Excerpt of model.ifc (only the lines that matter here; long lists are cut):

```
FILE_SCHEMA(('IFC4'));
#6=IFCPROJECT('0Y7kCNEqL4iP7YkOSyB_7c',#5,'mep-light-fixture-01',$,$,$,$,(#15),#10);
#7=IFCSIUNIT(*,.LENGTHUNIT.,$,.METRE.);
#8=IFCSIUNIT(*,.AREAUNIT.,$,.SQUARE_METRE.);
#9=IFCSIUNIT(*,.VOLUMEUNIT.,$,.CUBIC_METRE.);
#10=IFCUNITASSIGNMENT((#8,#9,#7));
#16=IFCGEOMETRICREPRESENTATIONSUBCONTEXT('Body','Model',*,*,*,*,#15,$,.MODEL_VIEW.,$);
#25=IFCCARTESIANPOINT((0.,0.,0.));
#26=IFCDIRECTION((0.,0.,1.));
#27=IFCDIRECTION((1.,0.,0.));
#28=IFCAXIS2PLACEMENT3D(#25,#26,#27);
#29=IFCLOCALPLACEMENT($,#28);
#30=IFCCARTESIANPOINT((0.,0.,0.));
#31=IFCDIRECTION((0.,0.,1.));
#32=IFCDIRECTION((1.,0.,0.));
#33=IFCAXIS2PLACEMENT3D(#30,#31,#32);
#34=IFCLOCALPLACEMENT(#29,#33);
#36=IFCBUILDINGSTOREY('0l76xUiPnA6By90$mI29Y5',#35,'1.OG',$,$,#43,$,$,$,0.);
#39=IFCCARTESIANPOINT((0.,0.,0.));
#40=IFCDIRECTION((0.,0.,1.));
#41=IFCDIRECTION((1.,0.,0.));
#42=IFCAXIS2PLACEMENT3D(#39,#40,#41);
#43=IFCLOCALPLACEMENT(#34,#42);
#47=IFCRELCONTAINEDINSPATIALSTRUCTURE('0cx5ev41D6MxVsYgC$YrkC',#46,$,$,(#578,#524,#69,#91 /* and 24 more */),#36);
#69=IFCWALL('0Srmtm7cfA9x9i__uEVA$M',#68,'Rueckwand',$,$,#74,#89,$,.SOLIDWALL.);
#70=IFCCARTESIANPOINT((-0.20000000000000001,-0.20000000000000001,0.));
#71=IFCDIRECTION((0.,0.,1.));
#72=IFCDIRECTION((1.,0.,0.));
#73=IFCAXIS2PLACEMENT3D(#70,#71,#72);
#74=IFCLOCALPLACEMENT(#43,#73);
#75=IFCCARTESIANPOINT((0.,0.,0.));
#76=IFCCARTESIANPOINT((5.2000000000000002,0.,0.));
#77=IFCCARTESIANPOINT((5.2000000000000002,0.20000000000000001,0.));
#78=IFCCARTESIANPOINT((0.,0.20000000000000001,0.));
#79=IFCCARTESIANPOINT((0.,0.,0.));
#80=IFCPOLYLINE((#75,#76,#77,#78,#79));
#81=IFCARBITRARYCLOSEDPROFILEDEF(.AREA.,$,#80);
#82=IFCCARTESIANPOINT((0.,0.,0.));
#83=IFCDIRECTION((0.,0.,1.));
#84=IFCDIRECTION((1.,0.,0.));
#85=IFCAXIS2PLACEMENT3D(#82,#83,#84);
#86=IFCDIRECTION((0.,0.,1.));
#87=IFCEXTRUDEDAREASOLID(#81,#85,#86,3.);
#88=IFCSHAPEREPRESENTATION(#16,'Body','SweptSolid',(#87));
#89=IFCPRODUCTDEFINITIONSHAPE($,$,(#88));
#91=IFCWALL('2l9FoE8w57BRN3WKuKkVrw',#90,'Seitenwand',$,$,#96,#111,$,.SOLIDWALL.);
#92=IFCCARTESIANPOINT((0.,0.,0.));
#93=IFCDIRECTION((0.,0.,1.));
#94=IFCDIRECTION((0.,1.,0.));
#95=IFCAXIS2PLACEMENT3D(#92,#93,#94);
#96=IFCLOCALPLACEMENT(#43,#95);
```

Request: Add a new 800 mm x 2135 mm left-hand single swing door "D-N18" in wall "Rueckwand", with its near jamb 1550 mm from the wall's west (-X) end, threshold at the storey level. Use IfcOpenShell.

```python
import numpy as np
import ifcopenshell
import ifcopenshell.api.feature
import ifcopenshell.api.geometry
import ifcopenshell.api.root
import ifcopenshell.api.spatial
import ifcopenshell.geom
import ifcopenshell.util.element
import ifcopenshell.util.placement
import ifcopenshell.util.representation
import ifcopenshell.util.shape
import ifcopenshell.util.unit

model = ifcopenshell.open("model.ifc")
unit_scale = ifcopenshell.util.unit.calculate_unit_scale(model)
settings = ifcopenshell.geom.settings()


def volume(element):
    """Net volume in cubic metres, openings subtracted."""
    shape = ifcopenshell.geom.create_shape(settings, element)
    return ifcopenshell.util.shape.get_volume(shape.geometry)


wall = model.by_guid("0Srmtm7cfA9x9i__uEVA$M")
storey = ifcopenshell.util.element.get_container(wall, ifc_class="IfcBuildingStorey")
context = ifcopenshell.util.representation.get_context(model, "Model", "Body", "MODEL_VIEW")
before = volume(wall)

width, height, from_end, sill = 0.8, 2.135, 1.55, 0.0  # metres

# The wall runs along its own X axis, and the end named is its -X end.
wall_shape = ifcopenshell.geom.create_shape(settings, wall)
x, y, z = ifcopenshell.util.shape.get_vertices(wall_shape.geometry).T
start = x.min() + from_end
face, thickness = float(y.min()), float(y.max() - y.min())
wall_matrix = ifcopenshell.util.placement.get_local_placement(wall.ObjectPlacement)
level = ifcopenshell.util.placement.get_local_placement(storey.ObjectPlacement)[2, 3]


def in_wall(x, y):
    """Placement at x, y metres in the wall's axes, at sill height."""
    matrix = wall_matrix.copy()
    matrix[:, 3] = wall_matrix @ np.array([x / unit_scale, y / unit_scale, 0.0, 1.0])
    matrix[2, 3] = level + sill / unit_scale
    return matrix


# Opening: a box that overshoots both wall faces by 50 mm.
opening = ifcopenshell.api.root.create_entity(model, ifc_class="IfcOpeningElement", predefined_type="OPENING")
box = ifcopenshell.api.geometry.add_wall_representation(
    model, context=context, length=width, height=height, thickness=thickness + 0.1
)
ifcopenshell.api.geometry.assign_representation(model, product=opening, representation=box)
ifcopenshell.api.geometry.edit_object_placement(model, product=opening, matrix=in_wall(start, face - 0.05), is_si=False)
ifcopenshell.api.feature.add_feature(model, feature=opening, element=wall)

door = ifcopenshell.api.root.create_entity(model, ifc_class="IfcDoor", name="D-N18", predefined_type="DOOR")
door.OverallWidth, door.OverallHeight = width / unit_scale, height / unit_scale
door.OperationType = "SINGLE_SWING_LEFT"
body = ifcopenshell.api.geometry.add_door_representation(
    model,
    context=context,
    overall_width=door.OverallWidth,
    overall_height=door.OverallHeight,
    operation_type="SINGLE_SWING_LEFT",
    lining_properties={"LiningDepth": thickness / unit_scale, "ThresholdDepth": thickness / unit_scale},
)
ifcopenshell.api.geometry.assign_representation(model, product=door, representation=body)
ifcopenshell.api.spatial.assign_container(model, products=[door], relating_structure=storey)
ifcopenshell.api.feature.add_filling(model, opening=opening, element=door)

# The lining spans the wall, so the door starts at the wall face.
ifcopenshell.api.geometry.edit_object_placement(model, product=door, matrix=in_wall(start, face), is_si=False)

after = volume(wall)

print(f"wall volume {before:.3f} -> {after:.3f} m3")

model.write("model_edited.ifc")
```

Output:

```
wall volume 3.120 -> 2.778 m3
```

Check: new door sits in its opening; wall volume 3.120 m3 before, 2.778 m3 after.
